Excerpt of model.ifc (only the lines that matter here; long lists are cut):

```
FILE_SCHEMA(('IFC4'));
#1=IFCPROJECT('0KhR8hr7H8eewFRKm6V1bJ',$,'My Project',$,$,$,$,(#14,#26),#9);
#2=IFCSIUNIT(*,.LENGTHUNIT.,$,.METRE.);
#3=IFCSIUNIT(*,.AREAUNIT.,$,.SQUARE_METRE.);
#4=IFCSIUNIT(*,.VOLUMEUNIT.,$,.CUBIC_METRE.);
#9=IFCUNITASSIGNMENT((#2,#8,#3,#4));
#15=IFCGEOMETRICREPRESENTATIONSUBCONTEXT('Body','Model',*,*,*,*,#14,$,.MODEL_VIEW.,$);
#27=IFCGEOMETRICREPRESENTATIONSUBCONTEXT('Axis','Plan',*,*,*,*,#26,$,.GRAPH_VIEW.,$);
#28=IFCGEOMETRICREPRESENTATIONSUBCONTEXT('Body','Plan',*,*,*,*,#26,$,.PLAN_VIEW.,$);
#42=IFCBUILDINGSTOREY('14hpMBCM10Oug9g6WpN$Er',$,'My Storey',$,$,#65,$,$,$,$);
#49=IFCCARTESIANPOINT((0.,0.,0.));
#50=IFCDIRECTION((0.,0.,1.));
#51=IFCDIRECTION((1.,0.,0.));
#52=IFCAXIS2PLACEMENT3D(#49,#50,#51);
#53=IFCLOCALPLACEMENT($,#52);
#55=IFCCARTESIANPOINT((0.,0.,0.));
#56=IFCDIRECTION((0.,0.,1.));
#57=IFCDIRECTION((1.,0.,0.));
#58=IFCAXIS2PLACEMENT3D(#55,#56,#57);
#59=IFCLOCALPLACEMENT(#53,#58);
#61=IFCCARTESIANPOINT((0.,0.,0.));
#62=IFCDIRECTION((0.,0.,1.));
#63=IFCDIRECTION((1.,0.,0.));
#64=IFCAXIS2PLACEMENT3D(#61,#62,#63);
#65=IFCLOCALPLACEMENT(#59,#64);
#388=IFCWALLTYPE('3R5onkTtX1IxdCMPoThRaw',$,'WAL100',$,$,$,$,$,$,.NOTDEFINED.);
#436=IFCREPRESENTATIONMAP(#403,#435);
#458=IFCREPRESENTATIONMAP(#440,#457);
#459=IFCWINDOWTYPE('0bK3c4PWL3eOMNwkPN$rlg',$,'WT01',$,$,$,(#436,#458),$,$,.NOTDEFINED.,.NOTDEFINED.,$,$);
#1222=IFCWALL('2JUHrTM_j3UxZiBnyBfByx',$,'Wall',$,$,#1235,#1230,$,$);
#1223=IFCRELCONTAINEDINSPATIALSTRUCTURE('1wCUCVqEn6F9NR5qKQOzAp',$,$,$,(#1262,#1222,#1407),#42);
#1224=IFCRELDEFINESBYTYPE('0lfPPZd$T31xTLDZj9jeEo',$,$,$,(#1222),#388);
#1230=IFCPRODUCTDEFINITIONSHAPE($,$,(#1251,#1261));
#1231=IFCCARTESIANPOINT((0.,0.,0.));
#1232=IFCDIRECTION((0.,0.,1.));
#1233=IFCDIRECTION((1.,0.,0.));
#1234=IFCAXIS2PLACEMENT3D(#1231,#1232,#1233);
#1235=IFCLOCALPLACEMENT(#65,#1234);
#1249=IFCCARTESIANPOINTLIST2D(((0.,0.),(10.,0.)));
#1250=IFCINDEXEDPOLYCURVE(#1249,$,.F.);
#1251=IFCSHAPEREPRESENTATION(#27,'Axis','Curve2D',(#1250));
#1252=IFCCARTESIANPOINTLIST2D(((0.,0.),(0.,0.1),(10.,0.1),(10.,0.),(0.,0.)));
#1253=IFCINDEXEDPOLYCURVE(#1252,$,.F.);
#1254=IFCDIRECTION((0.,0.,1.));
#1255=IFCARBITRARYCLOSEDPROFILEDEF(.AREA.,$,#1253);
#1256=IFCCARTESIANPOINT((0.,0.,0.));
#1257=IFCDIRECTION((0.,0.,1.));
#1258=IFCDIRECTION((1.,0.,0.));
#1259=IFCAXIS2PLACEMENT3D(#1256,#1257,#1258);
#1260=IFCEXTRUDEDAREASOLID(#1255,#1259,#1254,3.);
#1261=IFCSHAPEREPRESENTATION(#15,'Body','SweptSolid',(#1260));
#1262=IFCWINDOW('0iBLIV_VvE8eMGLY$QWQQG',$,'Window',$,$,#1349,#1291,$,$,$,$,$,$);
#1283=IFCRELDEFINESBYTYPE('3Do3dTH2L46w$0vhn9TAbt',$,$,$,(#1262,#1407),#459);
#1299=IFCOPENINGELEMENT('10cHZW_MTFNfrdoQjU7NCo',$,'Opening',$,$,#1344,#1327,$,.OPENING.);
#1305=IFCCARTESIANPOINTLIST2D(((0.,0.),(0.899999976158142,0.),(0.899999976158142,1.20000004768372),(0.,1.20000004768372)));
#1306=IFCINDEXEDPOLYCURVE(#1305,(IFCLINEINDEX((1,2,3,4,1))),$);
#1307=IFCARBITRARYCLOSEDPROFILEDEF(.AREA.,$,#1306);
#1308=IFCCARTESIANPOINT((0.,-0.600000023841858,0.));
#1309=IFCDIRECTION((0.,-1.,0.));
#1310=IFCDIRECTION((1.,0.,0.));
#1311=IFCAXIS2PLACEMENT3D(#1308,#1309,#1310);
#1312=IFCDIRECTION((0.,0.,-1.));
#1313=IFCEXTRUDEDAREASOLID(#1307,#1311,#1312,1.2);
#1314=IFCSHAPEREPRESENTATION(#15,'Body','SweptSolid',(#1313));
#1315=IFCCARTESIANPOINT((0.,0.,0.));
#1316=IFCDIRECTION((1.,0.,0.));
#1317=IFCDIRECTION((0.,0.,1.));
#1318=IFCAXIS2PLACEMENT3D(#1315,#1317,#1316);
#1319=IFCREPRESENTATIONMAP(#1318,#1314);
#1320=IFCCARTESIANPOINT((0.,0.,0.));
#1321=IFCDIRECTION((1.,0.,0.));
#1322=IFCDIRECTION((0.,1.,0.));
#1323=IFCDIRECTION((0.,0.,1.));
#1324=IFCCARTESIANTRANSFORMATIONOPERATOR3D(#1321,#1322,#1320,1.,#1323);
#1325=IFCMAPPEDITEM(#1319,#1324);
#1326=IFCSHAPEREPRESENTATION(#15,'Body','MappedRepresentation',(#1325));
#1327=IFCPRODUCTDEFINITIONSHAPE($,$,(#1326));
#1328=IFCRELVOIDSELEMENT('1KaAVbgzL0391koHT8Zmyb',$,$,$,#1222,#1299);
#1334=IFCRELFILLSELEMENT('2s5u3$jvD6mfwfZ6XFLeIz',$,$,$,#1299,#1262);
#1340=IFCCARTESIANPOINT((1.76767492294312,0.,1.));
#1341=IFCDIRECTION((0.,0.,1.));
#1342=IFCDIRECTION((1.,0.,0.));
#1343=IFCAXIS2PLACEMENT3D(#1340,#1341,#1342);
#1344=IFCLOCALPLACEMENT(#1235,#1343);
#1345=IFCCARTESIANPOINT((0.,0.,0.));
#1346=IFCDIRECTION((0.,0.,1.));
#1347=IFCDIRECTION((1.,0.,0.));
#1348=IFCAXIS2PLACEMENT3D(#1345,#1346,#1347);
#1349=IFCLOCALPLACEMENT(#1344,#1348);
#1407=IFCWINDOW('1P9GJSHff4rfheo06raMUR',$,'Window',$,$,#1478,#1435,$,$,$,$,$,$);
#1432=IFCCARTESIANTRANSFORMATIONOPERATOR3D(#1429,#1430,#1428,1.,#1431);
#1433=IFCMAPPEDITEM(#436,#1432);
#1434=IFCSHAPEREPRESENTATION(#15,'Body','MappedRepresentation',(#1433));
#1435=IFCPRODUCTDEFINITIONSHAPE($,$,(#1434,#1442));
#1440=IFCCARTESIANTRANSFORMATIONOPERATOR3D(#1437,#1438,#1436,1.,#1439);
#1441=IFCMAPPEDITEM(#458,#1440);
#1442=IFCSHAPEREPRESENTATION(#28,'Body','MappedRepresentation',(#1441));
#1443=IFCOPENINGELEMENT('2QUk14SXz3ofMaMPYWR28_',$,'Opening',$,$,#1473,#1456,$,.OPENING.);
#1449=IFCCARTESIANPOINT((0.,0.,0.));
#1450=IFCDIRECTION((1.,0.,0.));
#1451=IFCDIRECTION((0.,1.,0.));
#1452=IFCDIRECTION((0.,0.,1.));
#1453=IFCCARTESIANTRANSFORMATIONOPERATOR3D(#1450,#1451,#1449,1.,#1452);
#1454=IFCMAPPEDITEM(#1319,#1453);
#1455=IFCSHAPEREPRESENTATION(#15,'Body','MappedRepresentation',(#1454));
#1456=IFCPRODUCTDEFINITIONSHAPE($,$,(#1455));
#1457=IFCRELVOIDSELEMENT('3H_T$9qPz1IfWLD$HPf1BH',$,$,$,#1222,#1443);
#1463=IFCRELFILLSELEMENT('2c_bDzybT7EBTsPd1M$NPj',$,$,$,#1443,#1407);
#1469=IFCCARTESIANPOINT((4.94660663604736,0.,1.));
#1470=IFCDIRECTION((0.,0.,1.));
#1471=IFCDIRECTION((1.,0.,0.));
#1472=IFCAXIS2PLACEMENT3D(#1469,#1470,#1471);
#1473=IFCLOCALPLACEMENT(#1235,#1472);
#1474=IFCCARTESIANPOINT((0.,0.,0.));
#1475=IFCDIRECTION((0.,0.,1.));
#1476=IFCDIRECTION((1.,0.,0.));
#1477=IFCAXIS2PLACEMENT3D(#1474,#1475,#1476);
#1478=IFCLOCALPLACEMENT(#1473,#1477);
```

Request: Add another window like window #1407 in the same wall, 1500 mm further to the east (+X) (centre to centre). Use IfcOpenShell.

```python
import ifcopenshell
import ifcopenshell.api.feature
import ifcopenshell.api.geometry
import ifcopenshell.api.root
import ifcopenshell.geom
import ifcopenshell.util.element
import ifcopenshell.util.placement
import ifcopenshell.util.shape

model = ifcopenshell.open("model.ifc")
settings = ifcopenshell.geom.settings()


def volume(element):
    """Net volume in cubic metres, openings subtracted."""
    shape = ifcopenshell.geom.create_shape(settings, element)
    return ifcopenshell.util.shape.get_volume(shape.geometry)


window = model.by_guid("1P9GJSHff4rfheo06raMUR")
opening = window.FillsVoids[0].RelatingOpeningElement
wall = opening.VoidsElements[0].RelatingBuildingElement
before = volume(wall)
shift = ifcopenshell.util.placement.get_local_placement(wall.ObjectPlacement)[:3, 0] * 1.5

# copy_class copies the void relationship, type, container and properties, but no geometry.
new_opening = ifcopenshell.api.root.copy_class(model, product=opening)
new_opening.Representation = ifcopenshell.util.element.copy_deep(
    model, opening.Representation, exclude=["IfcGeometricRepresentationContext", "IfcRepresentationMap"]
)
new_window = ifcopenshell.api.root.copy_class(model, product=window)
new_window.Representation = ifcopenshell.util.element.copy_deep(
    model, window.Representation, exclude=["IfcGeometricRepresentationContext", "IfcRepresentationMap"]
)
ifcopenshell.api.feature.add_filling(model, opening=new_opening, element=new_window)

for old, new in ((opening, new_opening), (window, new_window)):
    matrix = ifcopenshell.util.placement.get_local_placement(old.ObjectPlacement)
    matrix[:3, 3] += shift
    ifcopenshell.api.geometry.edit_object_placement(model, product=new, matrix=matrix, is_si=False)

after = volume(wall)

print(f"wall volume {before:.3f} -> {after:.3f} m3")

model.write("model_edited.ifc")
```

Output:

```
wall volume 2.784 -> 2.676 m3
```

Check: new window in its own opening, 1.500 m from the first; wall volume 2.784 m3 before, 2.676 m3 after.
